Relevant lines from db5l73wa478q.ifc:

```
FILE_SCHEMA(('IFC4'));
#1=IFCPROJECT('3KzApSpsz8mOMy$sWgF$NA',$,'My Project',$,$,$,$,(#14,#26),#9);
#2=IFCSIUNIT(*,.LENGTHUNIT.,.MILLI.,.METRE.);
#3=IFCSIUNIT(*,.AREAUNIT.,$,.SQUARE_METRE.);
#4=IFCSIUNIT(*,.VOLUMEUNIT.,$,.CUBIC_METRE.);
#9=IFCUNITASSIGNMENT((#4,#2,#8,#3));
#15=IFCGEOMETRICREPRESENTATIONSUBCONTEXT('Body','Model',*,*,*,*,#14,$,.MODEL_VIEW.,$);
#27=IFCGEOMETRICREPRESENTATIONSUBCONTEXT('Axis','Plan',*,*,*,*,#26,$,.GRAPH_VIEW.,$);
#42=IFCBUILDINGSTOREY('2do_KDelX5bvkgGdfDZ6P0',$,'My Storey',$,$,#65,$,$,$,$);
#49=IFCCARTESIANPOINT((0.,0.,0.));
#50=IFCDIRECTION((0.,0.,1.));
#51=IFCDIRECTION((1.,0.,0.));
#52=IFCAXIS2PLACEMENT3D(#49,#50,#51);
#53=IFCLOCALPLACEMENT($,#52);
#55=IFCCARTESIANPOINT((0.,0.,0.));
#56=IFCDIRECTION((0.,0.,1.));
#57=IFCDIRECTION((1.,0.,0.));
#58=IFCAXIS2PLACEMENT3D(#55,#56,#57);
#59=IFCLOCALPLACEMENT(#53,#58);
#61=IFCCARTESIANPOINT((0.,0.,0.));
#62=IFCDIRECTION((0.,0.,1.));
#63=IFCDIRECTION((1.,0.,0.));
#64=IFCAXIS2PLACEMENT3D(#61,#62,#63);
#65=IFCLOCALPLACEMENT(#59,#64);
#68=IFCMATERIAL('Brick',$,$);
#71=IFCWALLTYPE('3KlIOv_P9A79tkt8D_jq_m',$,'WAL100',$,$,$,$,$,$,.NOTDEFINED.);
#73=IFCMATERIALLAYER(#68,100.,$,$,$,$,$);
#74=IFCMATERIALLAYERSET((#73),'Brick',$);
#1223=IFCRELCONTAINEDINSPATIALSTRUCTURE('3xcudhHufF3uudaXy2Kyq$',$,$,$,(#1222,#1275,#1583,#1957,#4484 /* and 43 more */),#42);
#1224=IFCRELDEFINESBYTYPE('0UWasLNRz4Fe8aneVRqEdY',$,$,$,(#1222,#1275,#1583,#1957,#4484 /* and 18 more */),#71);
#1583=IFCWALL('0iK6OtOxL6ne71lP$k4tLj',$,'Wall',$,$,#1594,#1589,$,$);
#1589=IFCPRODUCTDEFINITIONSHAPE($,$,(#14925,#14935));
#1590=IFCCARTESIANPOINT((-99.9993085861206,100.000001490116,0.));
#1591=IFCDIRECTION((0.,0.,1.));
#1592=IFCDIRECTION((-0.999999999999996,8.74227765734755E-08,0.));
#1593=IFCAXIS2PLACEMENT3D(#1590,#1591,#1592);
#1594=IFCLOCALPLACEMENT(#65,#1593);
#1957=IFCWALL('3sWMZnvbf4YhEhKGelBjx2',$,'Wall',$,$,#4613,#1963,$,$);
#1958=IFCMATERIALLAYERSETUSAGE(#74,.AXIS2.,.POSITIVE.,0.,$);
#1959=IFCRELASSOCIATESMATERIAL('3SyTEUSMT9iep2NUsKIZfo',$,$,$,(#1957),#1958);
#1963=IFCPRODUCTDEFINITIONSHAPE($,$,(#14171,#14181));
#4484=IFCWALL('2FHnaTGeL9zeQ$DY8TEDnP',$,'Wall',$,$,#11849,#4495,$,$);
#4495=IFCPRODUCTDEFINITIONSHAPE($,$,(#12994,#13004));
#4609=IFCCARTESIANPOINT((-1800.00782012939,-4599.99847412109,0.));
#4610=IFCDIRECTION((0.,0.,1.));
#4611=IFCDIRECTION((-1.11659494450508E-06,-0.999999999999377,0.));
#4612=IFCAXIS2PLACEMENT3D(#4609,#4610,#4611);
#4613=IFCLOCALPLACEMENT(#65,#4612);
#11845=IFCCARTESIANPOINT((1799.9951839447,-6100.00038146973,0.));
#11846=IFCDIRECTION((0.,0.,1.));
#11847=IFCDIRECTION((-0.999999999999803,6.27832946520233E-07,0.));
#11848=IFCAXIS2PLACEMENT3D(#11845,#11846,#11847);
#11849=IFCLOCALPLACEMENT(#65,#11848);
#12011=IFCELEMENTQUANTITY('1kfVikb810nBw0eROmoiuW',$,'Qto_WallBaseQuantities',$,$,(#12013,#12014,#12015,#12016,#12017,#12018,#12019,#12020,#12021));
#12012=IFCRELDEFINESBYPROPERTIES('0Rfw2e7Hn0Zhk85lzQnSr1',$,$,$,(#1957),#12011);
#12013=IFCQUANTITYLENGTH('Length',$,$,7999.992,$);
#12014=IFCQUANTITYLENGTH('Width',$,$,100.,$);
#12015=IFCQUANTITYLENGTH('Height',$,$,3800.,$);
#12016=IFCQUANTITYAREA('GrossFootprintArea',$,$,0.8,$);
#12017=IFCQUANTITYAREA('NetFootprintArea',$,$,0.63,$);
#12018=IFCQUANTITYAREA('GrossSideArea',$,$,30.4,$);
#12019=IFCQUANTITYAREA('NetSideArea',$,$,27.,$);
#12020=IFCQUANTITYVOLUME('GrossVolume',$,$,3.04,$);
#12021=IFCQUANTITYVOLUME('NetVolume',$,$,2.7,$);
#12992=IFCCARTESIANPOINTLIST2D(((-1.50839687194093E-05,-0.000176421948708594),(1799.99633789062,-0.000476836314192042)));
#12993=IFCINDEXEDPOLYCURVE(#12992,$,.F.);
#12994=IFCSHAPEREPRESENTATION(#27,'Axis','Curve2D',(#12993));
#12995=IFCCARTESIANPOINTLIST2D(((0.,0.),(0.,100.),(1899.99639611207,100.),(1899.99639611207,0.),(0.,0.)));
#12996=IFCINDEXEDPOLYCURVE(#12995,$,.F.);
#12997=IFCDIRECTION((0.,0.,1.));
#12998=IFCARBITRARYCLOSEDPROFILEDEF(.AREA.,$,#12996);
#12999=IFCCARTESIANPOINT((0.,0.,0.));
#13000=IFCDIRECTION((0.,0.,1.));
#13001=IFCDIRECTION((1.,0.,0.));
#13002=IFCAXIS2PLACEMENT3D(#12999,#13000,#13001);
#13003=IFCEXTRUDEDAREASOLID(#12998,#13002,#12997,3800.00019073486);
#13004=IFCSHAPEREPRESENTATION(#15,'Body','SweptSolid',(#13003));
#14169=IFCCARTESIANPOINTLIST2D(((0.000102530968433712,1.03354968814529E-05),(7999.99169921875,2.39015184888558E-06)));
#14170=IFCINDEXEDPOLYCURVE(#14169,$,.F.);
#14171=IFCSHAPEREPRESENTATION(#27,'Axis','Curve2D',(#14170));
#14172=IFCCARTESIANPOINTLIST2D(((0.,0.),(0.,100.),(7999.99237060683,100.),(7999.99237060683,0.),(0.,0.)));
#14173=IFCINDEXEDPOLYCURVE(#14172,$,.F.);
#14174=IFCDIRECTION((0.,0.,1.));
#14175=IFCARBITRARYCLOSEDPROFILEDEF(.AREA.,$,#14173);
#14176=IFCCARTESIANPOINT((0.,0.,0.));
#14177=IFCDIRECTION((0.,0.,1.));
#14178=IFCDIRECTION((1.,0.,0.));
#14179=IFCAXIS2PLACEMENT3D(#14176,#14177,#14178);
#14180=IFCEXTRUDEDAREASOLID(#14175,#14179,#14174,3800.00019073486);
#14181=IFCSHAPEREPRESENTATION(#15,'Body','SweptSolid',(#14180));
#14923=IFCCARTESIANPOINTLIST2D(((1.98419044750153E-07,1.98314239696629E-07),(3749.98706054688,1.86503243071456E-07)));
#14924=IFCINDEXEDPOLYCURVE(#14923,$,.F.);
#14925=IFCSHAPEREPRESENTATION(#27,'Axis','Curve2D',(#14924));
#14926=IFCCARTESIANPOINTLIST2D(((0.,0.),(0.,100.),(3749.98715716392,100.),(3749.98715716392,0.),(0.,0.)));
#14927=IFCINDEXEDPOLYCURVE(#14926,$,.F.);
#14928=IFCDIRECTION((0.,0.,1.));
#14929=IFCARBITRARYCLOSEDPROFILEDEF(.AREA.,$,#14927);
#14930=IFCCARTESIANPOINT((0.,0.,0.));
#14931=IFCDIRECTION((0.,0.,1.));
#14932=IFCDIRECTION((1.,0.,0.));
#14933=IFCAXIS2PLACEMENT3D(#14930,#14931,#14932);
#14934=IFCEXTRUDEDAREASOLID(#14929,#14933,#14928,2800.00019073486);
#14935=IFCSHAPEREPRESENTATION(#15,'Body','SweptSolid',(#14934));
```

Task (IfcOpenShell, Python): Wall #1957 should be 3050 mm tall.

```python
import ifcopenshell
import ifcopenshell.api.pset
import ifcopenshell.geom
import ifcopenshell.util.element
import ifcopenshell.util.representation
import ifcopenshell.util.shape
import ifcopenshell.util.unit

model = ifcopenshell.open("db5l73wa478q.ifc")
unit_scale = ifcopenshell.util.unit.calculate_unit_scale(model)
area_scale = ifcopenshell.util.unit.calculate_unit_scale(model, "AREAUNIT")
volume_scale = ifcopenshell.util.unit.calculate_unit_scale(model, "VOLUMEUNIT")
settings = ifcopenshell.geom.settings()


def volume(element):
    """Net volume in cubic metres, openings subtracted."""
    shape = ifcopenshell.geom.create_shape(settings, element)
    return ifcopenshell.util.shape.get_volume(shape.geometry)


wall = model.by_id(1957)
before = volume(wall)

body = ifcopenshell.util.representation.get_representation(wall, "Model", "Body")
solid = body.Items[0]
old_height = solid.Depth
solid.Depth = 3.05 / unit_scale
after = volume(wall)
thickness = 0.1  # wall thickness in metres

# Update the stored height, areas and volumes.
qto = model.by_id(ifcopenshell.util.element.get_pset(wall, "Qto_WallBaseQuantities", should_inherit=False)["id"])
ifcopenshell.api.pset.edit_qto(model, qto=qto, properties={
    "Height": solid.Depth,
    "GrossSideArea": ifcopenshell.util.element.get_pset(wall, "Qto_WallBaseQuantities", "GrossSideArea") * solid.Depth / old_height,
    "NetSideArea": after / thickness / area_scale,
    "GrossVolume": ifcopenshell.util.element.get_pset(wall, "Qto_WallBaseQuantities", "GrossVolume") * solid.Depth / old_height,
    "NetVolume": after / volume_scale,
})

print(f"height {old_height:g} -> {solid.Depth:g}, volume {before:.3f} -> {after:.3f} m3")

model.write("db5l73wa478q_rev.ifc")
```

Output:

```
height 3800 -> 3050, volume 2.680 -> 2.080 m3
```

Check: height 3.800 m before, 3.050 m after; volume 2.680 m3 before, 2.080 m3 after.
